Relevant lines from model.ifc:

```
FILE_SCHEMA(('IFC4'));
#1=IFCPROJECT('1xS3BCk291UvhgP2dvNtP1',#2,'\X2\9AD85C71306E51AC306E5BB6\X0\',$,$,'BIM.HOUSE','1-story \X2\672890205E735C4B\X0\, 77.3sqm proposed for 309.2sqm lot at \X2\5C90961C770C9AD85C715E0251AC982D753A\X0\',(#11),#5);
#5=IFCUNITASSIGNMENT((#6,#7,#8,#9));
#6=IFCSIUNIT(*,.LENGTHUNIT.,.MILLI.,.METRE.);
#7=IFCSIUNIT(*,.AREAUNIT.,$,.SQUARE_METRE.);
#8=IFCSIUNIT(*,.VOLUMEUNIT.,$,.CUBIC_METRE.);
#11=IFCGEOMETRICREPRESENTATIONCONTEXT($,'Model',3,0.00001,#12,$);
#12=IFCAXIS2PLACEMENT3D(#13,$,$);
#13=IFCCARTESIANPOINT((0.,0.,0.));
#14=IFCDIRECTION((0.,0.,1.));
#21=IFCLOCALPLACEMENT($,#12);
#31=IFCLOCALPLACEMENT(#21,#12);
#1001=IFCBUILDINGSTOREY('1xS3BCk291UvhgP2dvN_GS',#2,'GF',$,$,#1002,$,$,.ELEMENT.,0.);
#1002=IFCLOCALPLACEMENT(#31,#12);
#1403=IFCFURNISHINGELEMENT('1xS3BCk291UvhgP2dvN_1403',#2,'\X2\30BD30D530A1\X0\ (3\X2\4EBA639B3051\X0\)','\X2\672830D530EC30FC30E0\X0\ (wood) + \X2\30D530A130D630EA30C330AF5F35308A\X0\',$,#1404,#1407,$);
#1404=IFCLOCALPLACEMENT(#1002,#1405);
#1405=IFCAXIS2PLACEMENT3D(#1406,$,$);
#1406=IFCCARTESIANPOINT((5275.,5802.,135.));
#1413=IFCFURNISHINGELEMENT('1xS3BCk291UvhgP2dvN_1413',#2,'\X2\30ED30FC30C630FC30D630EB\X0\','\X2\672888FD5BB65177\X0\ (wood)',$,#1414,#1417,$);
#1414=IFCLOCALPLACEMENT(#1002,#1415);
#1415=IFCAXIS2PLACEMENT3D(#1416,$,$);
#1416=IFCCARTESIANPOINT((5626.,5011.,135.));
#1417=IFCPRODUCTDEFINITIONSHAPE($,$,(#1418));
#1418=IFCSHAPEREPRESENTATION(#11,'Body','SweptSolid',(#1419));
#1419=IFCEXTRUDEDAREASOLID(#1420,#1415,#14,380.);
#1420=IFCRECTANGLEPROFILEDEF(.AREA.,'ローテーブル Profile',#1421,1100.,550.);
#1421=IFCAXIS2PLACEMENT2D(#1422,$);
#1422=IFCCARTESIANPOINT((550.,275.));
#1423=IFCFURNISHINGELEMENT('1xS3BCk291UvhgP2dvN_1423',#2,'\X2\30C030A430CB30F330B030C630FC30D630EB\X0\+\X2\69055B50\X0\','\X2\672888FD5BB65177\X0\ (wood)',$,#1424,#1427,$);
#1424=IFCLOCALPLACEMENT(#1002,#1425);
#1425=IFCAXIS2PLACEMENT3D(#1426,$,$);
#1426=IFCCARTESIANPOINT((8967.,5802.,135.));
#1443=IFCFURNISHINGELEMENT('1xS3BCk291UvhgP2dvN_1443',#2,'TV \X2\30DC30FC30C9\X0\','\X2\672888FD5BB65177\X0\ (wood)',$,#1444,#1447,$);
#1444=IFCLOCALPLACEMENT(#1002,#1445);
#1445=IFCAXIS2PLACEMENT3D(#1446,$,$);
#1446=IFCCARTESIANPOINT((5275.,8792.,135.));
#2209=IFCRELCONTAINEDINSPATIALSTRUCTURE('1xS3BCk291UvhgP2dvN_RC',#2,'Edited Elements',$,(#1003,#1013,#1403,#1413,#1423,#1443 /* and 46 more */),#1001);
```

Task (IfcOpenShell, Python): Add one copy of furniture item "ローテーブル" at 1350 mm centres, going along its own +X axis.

```python
import ifcopenshell
import ifcopenshell.api.geometry
import ifcopenshell.api.root
import ifcopenshell.util.element
import ifcopenshell.util.placement
import ifcopenshell.util.unit

model = ifcopenshell.open("model.ifc")
unit_scale = ifcopenshell.util.unit.calculate_unit_scale(model)


def reuse_history(source, copy):
    """copy_class also copies each property set's owner history, people and application; keep the originals."""
    for rel in copy.IsDefinedBy:
        if rel.is_a("IfcRelDefinesByProperties") and (history := rel.RelatingPropertyDefinition.OwnerHistory):
            rel.RelatingPropertyDefinition.OwnerHistory = source.OwnerHistory
            ifcopenshell.util.element.remove_deep2(model, history)


source = model.by_guid("1xS3BCk291UvhgP2dvN_1413")
base = ifcopenshell.util.placement.get_local_placement(source.ObjectPlacement)
step = base[:3, 0] * 1.35 / unit_scale

for i in range(1, 2):
    copy = ifcopenshell.api.root.copy_class(model, product=source)
    copy.Representation = ifcopenshell.util.element.copy_deep(
        model, source.Representation, exclude=["IfcGeometricRepresentationContext", "IfcRepresentationMap"]
    )
    reuse_history(source, copy)
    matrix = base.copy()
    matrix[:3, 3] += i * step
    print("added at", matrix[:3, 3].round(3) + 0.0)
    ifcopenshell.api.geometry.edit_object_placement(model, product=copy, matrix=matrix, is_si=False)

model.write("model-out.ifc")
```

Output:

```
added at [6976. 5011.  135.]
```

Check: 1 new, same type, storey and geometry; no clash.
